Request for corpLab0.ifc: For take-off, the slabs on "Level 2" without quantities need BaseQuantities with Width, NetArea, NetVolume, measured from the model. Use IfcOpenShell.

First a look at what the model holds.

```python
import ifcopenshell
import ifcopenshell.util.element
import ifcopenshell.util.unit

model = ifcopenshell.open("corpLab0.ifc")
print(model.schema)
for unit_type in ("LENGTHUNIT", "AREAUNIT", "VOLUMEUNIT"):
    print(unit_type, ifcopenshell.util.unit.calculate_unit_scale(model, unit_type))
storey = next(s for s in model.by_type("IfcBuildingStorey") if s.Name == "Level 2")
slabs = [e for e in ifcopenshell.util.element.get_decomposition(storey) if e.is_a("IfcSlab")]
for e in sorted(slabs, key=lambda e: e.id()):
    print(e.id(), e.is_a(), e.Name, list(ifcopenshell.util.element.get_psets(e, qtos_only=True)), sep=" | ")
```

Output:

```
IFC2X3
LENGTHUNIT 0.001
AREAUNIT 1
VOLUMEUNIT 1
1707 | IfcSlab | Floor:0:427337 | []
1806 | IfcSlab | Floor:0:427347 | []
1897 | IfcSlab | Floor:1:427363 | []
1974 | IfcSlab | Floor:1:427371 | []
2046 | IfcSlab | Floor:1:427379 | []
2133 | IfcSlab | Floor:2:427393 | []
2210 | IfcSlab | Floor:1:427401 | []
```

```python
import ifcopenshell
import ifcopenshell.api.pset
import ifcopenshell.geom
import ifcopenshell.util.element
import ifcopenshell.util.shape
import ifcopenshell.util.unit

model = ifcopenshell.open("corpLab0.ifc")
unit_scale = ifcopenshell.util.unit.calculate_unit_scale(model)
area_scale = ifcopenshell.util.unit.calculate_unit_scale(model, "AREAUNIT")
volume_scale = ifcopenshell.util.unit.calculate_unit_scale(model, "VOLUMEUNIT")
settings = ifcopenshell.geom.settings()

storey = next(s for s in model.by_type("IfcBuildingStorey") if s.Name == "Level 2")
slabs = [e for e in ifcopenshell.util.element.get_decomposition(storey) if e.is_a("IfcSlab")]

for e in sorted(slabs, key=lambda e: e.id()):
    if ifcopenshell.util.element.get_psets(e, qtos_only=True, should_inherit=False):
        continue
    # Geometry comes back in metres, in the element's own axes.
    shape = ifcopenshell.geom.create_shape(settings, e)
    values = {
        "Width": ifcopenshell.util.shape.get_z(shape.geometry) / unit_scale,
        "NetArea": ifcopenshell.util.shape.get_footprint_area(shape.geometry) / area_scale,
        "NetVolume": ifcopenshell.util.shape.get_volume(shape.geometry) / volume_scale,
    }
    qto = ifcopenshell.api.pset.add_qto(model, product=e, name="BaseQuantities")
    ifcopenshell.api.pset.edit_qto(model, qto=qto, properties=values)
    print(e.id(), {k: round(v, 3) for k, v in values.items()})

model.write("corpLab0_updated.ifc")
```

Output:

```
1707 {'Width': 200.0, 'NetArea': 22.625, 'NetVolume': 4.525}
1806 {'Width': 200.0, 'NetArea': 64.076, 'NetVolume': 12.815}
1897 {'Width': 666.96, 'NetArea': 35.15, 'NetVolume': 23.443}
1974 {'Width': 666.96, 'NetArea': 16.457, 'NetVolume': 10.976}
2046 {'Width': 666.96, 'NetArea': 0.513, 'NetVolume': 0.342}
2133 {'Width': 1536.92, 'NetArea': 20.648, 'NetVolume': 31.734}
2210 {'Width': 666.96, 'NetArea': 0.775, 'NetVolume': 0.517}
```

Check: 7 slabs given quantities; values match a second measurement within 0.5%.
